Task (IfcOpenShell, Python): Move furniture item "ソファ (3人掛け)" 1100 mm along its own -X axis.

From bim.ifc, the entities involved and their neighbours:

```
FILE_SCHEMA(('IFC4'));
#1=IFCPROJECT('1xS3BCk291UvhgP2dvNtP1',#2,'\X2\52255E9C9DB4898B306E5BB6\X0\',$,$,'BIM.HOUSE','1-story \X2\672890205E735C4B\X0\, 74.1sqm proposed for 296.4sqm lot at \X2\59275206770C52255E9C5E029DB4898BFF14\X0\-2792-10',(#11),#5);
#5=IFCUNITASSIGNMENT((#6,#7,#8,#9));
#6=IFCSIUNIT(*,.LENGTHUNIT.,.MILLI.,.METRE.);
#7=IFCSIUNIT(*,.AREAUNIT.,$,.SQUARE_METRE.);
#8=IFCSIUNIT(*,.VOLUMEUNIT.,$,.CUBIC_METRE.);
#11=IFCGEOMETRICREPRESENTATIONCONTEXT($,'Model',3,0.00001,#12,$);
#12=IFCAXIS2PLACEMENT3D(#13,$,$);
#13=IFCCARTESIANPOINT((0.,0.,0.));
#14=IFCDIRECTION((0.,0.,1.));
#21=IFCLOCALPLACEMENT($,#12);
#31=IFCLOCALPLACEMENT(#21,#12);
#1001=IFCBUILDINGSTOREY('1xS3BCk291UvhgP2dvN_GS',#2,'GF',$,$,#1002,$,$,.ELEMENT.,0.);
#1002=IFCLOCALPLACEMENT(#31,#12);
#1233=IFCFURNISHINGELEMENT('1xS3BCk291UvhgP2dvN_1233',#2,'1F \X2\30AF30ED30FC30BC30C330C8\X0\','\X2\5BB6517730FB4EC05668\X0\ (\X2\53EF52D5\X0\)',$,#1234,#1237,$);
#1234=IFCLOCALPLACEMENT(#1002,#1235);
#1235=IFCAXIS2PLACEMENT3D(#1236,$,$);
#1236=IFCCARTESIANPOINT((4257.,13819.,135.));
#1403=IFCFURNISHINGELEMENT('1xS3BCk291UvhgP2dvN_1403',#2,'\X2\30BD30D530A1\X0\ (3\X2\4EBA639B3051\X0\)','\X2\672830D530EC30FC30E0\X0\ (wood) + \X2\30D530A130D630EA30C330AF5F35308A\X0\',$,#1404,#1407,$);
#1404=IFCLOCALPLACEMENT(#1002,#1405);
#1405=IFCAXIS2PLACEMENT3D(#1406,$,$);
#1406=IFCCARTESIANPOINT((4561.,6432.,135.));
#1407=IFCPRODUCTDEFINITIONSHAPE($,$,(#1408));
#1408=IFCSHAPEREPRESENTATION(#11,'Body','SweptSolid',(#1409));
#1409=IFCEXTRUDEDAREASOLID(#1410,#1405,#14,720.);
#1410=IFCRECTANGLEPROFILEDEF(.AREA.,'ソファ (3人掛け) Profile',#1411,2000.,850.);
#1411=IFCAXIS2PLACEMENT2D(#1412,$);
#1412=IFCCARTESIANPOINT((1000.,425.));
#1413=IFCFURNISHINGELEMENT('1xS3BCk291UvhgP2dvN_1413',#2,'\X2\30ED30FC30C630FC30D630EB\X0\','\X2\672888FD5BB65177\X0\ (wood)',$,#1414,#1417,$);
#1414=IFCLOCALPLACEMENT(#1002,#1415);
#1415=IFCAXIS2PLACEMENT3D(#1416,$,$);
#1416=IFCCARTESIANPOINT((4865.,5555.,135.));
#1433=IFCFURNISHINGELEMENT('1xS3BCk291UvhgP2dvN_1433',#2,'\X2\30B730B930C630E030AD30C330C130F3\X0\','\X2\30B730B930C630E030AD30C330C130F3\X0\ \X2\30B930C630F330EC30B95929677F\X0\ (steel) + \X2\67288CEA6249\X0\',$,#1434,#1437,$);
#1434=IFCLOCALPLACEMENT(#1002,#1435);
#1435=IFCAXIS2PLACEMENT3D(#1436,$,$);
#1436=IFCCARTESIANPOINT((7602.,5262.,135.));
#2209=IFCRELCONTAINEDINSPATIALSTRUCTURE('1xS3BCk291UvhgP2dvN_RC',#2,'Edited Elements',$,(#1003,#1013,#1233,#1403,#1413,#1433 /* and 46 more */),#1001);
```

```python
import ifcopenshell
import ifcopenshell.api.geometry
import ifcopenshell.util.placement
import ifcopenshell.util.unit

model = ifcopenshell.open("bim.ifc")
unit_scale = ifcopenshell.util.unit.calculate_unit_scale(model)

item = model.by_id(1403)
matrix = ifcopenshell.util.placement.get_local_placement(item.ObjectPlacement)
matrix[:3, 3] -= matrix[:3, 0] * 1.1 / unit_scale
ifcopenshell.api.geometry.edit_object_placement(model, product=item, matrix=matrix, is_si=False)

print(ifcopenshell.util.placement.get_local_placement(item.ObjectPlacement).round(3) + 0.0)

model.write("bim_rev.ifc")
```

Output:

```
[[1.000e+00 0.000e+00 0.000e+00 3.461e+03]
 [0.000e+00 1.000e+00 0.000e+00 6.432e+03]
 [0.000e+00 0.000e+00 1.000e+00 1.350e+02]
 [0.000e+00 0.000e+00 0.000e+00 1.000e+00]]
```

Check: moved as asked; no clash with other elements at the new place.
